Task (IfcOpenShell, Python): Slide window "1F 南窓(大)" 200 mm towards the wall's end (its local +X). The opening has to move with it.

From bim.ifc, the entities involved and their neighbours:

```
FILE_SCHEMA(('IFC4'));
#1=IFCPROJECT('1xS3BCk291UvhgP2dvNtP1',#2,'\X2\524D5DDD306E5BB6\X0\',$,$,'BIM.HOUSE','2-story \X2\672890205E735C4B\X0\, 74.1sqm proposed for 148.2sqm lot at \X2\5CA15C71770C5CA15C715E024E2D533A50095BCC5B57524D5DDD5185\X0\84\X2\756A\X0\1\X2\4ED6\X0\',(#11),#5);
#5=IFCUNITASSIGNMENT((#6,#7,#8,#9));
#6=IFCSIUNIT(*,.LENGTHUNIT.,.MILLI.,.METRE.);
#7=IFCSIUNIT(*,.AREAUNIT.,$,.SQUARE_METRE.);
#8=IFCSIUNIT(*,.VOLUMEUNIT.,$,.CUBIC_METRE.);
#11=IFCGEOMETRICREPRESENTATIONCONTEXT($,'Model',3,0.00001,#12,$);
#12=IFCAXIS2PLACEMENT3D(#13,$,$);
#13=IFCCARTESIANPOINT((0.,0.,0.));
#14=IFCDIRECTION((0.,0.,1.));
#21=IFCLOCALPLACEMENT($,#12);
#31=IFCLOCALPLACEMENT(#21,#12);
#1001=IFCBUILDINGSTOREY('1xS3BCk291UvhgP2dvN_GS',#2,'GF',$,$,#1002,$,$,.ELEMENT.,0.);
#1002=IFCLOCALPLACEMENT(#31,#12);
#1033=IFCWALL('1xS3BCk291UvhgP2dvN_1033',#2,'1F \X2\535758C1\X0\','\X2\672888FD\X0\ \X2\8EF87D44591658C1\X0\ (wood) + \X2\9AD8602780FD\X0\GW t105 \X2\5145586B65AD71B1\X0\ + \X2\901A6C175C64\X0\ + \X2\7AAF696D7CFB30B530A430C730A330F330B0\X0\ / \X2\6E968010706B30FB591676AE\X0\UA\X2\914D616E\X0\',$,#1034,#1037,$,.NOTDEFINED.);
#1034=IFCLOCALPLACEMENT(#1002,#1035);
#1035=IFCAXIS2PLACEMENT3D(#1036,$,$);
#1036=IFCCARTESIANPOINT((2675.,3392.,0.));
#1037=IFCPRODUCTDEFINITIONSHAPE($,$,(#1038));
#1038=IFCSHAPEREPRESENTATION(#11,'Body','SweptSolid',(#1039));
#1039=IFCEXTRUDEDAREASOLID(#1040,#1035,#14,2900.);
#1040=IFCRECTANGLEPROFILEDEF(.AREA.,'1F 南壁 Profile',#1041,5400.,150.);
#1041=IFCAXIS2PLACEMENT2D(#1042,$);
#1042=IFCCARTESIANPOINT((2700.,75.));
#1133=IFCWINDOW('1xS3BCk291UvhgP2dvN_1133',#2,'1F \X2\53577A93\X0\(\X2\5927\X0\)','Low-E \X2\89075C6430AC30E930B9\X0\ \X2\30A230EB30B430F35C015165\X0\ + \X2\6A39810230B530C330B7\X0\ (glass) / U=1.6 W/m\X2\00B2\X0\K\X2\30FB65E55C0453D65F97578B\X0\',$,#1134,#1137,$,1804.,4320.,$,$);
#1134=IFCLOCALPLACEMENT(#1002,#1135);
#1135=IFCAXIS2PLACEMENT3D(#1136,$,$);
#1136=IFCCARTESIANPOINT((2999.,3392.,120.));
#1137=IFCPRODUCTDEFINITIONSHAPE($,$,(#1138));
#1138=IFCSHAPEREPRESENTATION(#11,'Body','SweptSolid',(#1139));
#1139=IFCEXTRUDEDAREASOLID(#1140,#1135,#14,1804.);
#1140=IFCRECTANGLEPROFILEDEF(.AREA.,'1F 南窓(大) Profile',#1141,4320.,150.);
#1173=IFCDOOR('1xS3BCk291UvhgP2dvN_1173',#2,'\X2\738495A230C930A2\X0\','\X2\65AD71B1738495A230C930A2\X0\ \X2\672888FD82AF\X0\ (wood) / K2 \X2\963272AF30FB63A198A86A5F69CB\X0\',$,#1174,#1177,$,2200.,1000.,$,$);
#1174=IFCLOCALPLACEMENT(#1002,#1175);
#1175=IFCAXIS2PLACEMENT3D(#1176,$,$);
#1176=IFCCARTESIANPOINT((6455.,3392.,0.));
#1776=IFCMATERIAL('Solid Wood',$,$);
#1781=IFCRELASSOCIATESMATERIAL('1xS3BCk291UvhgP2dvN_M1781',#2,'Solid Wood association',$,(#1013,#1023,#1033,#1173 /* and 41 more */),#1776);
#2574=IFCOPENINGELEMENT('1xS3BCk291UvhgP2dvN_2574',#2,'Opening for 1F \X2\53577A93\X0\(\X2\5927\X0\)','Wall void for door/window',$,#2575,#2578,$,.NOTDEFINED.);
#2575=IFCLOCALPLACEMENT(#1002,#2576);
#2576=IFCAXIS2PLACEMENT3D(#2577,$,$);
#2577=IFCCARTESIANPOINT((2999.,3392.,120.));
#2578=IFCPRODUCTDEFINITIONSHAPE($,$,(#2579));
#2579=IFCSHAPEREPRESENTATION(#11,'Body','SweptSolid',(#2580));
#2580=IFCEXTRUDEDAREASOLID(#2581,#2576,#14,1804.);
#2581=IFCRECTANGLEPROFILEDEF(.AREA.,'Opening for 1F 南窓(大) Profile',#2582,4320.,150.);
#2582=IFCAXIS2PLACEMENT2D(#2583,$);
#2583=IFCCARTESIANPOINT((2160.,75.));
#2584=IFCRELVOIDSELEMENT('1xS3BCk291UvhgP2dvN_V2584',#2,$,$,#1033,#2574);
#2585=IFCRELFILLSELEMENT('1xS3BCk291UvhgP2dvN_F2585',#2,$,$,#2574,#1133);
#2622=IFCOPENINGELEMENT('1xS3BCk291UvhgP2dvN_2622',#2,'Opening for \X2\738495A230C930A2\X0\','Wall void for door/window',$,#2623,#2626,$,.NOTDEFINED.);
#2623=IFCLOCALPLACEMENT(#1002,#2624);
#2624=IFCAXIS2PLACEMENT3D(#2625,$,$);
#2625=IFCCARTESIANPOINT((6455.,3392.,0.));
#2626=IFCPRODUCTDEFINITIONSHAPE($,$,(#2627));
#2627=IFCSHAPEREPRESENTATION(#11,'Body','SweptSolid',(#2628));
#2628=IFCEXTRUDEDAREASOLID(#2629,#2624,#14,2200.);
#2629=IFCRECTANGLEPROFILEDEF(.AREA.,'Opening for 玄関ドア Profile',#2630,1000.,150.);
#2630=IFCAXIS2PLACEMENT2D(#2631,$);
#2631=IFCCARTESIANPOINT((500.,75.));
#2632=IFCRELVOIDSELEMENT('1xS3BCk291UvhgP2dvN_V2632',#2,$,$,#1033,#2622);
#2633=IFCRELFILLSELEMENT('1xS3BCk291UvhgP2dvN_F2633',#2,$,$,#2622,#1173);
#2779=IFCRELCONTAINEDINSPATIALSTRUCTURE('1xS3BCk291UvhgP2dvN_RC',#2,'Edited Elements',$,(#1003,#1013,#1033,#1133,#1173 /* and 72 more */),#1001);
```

```python
import ifcopenshell
import ifcopenshell.api.geometry
import ifcopenshell.util.placement

model = ifcopenshell.open("bim.ifc")

window = model.by_guid("1xS3BCk291UvhgP2dvN_1133")
opening = window.FillsVoids[0].RelatingOpeningElement
wall = opening.VoidsElements[0].RelatingBuildingElement

wall_matrix = ifcopenshell.util.placement.get_local_placement(wall.ObjectPlacement)
shift = wall_matrix[:3, 0] * 200.0
before = ifcopenshell.util.placement.get_local_placement(window.ObjectPlacement)[:3, 3].copy()

# The window is not placed relative to its opening, so move both.
for product in (opening, window):
    matrix = ifcopenshell.util.placement.get_local_placement(product.ObjectPlacement)
    matrix[:3, 3] += shift
    ifcopenshell.api.geometry.edit_object_placement(model, product=product, matrix=matrix, is_si=False)

after = ifcopenshell.util.placement.get_local_placement(window.ObjectPlacement)[:3, 3]
print("window moved by", (after - before).round(3) + 0.0)

model.write("bim_rev.ifc")
```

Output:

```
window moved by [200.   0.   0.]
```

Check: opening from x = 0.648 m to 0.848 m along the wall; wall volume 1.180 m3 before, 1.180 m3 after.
